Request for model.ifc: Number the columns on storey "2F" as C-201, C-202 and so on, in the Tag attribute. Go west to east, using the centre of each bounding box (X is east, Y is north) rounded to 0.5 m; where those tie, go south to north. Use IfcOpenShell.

First a look at what the model holds.

```python
import ifcopenshell
import ifcopenshell.util.element
import ifcopenshell.util.placement

model = ifcopenshell.open("model.ifc")
print(model.schema)
storey = next(s for s in model.by_type("IfcBuildingStorey") if s.Name == "2F")
columns = [e for e in ifcopenshell.util.element.get_decomposition(storey) if e.is_a("IfcColumn")]
for e in sorted(columns, key=lambda e: e.id()):
    origin = ifcopenshell.util.placement.get_local_placement(e.ObjectPlacement)[:3, 3]
    print(e.id(), e.Tag, e.Name, origin.round(2) + 0.0, sep=" | ")
```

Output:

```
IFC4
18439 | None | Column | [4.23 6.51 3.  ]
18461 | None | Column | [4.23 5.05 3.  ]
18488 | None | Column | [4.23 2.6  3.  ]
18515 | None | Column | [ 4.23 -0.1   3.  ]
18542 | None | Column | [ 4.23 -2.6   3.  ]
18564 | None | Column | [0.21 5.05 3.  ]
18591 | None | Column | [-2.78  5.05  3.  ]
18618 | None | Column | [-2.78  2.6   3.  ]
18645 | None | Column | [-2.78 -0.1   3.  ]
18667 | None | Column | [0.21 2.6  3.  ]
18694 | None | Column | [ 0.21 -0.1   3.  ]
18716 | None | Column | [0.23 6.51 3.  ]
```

```python
import ifcopenshell
import ifcopenshell.geom
import ifcopenshell.util.element
import ifcopenshell.util.shape

model = ifcopenshell.open("model.ifc")
settings = ifcopenshell.geom.settings()
settings.set("use-world-coords", True)


def centre(element):
    shape = ifcopenshell.geom.create_shape(settings, element)
    return ifcopenshell.util.shape.get_bbox_centroid(shape.geometry)


storey = next(s for s in model.by_type("IfcBuildingStorey") if s.Name == "2F")
columns = [e for e in ifcopenshell.util.element.get_decomposition(storey) if e.is_a("IfcColumn")]

# Insertion points can sit at a corner or the storey origin, so sort by the geometry (in metres).
centres = {e: centre(e) for e in columns}
columns.sort(key=lambda e: (round(centres[e][0] / 0.5), centres[e][1]))

for i, e in enumerate(columns, start=1):
    number = f"C-2{i:02d}"
    e.Tag = number
    print(e.id(), number)

model.write("model-out.ifc")
```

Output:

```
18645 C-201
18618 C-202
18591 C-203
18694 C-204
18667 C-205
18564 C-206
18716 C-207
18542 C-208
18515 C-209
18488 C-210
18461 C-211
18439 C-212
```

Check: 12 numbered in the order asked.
